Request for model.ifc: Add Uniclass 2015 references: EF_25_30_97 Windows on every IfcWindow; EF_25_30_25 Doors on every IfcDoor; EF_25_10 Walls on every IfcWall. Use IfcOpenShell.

First a look at what the model holds.

```python
import ifcopenshell

model = ifcopenshell.open("model.ifc")
print(model.schema)
print("classifications:", [c.Name for c in model.by_type("IfcClassification")])
for ifc_class in ("IfcDoor", "IfcRoof", "IfcStair", "IfcWall", "IfcWindow"):
    print(ifc_class, len(model.by_type(ifc_class)))
```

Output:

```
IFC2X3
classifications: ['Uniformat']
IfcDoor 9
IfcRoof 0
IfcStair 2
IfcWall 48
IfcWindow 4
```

```python
import ifcopenshell
import ifcopenshell.api.classification

model = ifcopenshell.open("model.ifc")

# IFC2X3 requires Source and Edition and has no link from the project to the system.
system = model.create_entity("IfcClassification", Source="NBS", Edition="2015", Name="Uniclass 2015")

codes = {
    "IfcWindow": ("EF_25_30_97", "Windows"),
    "IfcDoor": ("EF_25_30_25", "Doors"),
    "IfcWall": ("EF_25_10", "Walls"),
}
for ifc_class, (code, name) in codes.items():
    products = model.by_type(ifc_class)
    ifcopenshell.api.classification.add_reference(
        model, products=products, classification=system, identification=code, name=name
    )
    print(code, len(products))

model.write("model-out.ifc")
```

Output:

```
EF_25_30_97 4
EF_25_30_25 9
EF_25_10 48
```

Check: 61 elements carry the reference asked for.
